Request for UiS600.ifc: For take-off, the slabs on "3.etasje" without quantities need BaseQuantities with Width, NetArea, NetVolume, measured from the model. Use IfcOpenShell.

First a look at what the model holds.

```python
import ifcopenshell
import ifcopenshell.util.element
import ifcopenshell.util.unit

model = ifcopenshell.open("UiS600.ifc")
print(model.schema)
for unit_type in ("LENGTHUNIT", "AREAUNIT", "VOLUMEUNIT"):
    print(unit_type, ifcopenshell.util.unit.calculate_unit_scale(model, unit_type))
storey = next(s for s in model.by_type("IfcBuildingStorey") if s.Name == "3.etasje")
slabs = [e for e in ifcopenshell.util.element.get_decomposition(storey) if e.is_a("IfcSlab")]
for e in sorted(slabs, key=lambda e: e.id()):
    print(e.id(), e.is_a(), e.Name, list(ifcopenshell.util.element.get_psets(e, qtos_only=True)), sep=" | ")
```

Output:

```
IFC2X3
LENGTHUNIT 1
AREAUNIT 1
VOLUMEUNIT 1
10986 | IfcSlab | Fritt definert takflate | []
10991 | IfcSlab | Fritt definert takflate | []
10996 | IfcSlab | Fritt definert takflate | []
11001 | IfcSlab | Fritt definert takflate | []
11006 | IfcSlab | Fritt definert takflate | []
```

```python
import ifcopenshell
import ifcopenshell.api.pset
import ifcopenshell.geom
import ifcopenshell.util.element
import ifcopenshell.util.shape
import ifcopenshell.util.unit

model = ifcopenshell.open("UiS600.ifc")
unit_scale = ifcopenshell.util.unit.calculate_unit_scale(model)
area_scale = ifcopenshell.util.unit.calculate_unit_scale(model, "AREAUNIT")
volume_scale = ifcopenshell.util.unit.calculate_unit_scale(model, "VOLUMEUNIT")
settings = ifcopenshell.geom.settings()

storey = next(s for s in model.by_type("IfcBuildingStorey") if s.Name == "3.etasje")
slabs = [e for e in ifcopenshell.util.element.get_decomposition(storey) if e.is_a("IfcSlab")]

for e in sorted(slabs, key=lambda e: e.id()):
    if ifcopenshell.util.element.get_psets(e, qtos_only=True, should_inherit=False):
        continue
    # Geometry comes back in metres, in the element's own axes.
    shape = ifcopenshell.geom.create_shape(settings, e)
    values = {
        "Width": ifcopenshell.util.shape.get_z(shape.geometry) / unit_scale,
        "NetArea": ifcopenshell.util.shape.get_footprint_area(shape.geometry) / area_scale,
        "NetVolume": ifcopenshell.util.shape.get_volume(shape.geometry) / volume_scale,
    }
    qto = ifcopenshell.api.pset.add_qto(model, product=e, name="BaseQuantities")
    ifcopenshell.api.pset.edit_qto(model, qto=qto, properties=values)
    print(e.id(), {k: round(v, 3) for k, v in values.items()})

model.write("UiS600_edited.ifc")
```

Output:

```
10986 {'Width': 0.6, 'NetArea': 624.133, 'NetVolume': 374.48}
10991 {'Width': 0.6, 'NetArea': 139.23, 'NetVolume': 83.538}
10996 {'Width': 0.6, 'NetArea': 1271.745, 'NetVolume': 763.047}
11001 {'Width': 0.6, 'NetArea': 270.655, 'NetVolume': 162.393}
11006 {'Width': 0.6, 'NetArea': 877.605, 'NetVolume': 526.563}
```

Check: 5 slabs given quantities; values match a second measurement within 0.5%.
